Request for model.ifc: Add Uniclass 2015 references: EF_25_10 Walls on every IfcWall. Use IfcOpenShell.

First a look at what the model holds.

```python
import ifcopenshell

model = ifcopenshell.open("model.ifc")
print(model.schema)
print("classifications:", [c.Name for c in model.by_type("IfcClassification")])
for ifc_class in ("IfcDoor", "IfcRoof", "IfcStair", "IfcWall", "IfcWindow"):
    print(ifc_class, len(model.by_type(ifc_class)))
```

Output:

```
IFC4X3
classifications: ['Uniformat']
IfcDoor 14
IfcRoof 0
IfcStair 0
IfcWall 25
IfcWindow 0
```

```python
import ifcopenshell
import ifcopenshell.api.classification

model = ifcopenshell.open("model.ifc")

system = ifcopenshell.api.classification.add_classification(model, classification="Uniclass 2015")

codes = {
    "IfcWall": ("EF_25_10", "Walls"),
}
for ifc_class, (code, name) in codes.items():
    products = model.by_type(ifc_class)
    ifcopenshell.api.classification.add_reference(
        model, products=products, classification=system, identification=code, name=name
    )
    print(code, len(products))

model.write("model_edited.ifc")
```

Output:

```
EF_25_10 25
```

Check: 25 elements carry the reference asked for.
